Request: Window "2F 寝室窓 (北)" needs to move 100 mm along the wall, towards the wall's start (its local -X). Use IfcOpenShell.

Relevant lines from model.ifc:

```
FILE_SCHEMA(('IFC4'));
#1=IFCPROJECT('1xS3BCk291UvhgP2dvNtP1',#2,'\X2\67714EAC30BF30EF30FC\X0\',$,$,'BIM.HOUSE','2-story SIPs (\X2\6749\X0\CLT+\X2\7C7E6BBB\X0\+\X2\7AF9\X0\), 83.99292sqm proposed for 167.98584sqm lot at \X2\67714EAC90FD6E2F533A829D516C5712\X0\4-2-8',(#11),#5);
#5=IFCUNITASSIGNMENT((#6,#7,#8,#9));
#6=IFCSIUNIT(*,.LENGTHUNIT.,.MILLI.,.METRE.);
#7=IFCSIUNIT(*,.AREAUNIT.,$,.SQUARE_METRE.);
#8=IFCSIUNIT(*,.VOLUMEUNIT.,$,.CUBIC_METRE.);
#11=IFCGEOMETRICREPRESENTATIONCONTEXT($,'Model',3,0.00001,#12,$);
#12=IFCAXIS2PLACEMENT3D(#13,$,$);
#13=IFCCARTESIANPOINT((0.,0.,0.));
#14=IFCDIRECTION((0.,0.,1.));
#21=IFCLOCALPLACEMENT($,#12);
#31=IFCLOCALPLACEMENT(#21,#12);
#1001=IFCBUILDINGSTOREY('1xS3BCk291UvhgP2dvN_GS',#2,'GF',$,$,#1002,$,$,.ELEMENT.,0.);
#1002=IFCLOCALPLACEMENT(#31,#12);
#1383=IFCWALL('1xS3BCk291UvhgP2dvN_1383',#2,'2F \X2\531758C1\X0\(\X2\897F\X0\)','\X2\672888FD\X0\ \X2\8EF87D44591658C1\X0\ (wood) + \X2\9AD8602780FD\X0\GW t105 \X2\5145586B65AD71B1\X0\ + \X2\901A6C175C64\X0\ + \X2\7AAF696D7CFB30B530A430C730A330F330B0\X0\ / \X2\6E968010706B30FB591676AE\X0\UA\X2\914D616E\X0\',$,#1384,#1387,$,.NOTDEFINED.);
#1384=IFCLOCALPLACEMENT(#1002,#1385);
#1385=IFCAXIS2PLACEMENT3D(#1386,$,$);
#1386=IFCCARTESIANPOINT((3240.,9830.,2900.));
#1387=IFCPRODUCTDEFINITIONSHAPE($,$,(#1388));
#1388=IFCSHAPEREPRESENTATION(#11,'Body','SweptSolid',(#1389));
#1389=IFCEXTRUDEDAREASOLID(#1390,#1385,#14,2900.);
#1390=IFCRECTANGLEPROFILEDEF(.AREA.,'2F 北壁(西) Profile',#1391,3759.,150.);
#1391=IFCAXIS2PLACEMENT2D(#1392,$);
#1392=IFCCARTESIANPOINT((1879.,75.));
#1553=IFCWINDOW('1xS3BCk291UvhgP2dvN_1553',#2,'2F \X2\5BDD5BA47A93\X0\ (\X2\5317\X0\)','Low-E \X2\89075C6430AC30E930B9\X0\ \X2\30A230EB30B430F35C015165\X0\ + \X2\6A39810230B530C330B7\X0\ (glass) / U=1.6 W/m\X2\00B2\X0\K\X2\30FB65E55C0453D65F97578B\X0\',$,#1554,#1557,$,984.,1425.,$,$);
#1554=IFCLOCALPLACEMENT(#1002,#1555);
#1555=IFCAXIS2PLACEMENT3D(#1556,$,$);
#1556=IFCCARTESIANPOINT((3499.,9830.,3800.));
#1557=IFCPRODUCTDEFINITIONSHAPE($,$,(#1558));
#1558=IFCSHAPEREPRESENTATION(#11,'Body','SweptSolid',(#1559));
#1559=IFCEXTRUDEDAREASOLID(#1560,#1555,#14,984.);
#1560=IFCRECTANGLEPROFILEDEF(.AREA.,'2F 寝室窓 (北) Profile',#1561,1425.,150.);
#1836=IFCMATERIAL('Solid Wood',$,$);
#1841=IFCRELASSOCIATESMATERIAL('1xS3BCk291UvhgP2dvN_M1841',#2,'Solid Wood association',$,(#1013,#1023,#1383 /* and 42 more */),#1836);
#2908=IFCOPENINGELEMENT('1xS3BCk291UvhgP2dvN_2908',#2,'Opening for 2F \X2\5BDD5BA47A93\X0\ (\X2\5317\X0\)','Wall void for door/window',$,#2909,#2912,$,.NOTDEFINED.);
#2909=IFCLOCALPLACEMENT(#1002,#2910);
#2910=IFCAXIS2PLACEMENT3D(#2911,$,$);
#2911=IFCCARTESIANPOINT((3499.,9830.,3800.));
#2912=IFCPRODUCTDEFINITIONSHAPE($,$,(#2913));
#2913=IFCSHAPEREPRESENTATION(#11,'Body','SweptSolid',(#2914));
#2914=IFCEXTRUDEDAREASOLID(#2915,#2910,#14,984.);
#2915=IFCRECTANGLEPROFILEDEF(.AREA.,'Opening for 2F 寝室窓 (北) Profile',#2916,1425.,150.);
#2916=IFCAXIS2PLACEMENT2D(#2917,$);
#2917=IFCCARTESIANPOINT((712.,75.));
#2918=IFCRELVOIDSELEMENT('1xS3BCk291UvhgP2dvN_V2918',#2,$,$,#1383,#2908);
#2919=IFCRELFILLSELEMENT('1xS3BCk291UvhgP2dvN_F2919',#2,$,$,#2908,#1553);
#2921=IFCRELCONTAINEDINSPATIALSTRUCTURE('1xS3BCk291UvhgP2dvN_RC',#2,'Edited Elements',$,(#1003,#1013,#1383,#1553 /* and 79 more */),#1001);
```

```python
import ifcopenshell
import ifcopenshell.api.geometry
import ifcopenshell.util.placement

model = ifcopenshell.open("model.ifc")

window = model.by_id(1553)
opening = window.FillsVoids[0].RelatingOpeningElement
wall = opening.VoidsElements[0].RelatingBuildingElement

wall_matrix = ifcopenshell.util.placement.get_local_placement(wall.ObjectPlacement)
shift = wall_matrix[:3, 0] * -100.0
before = ifcopenshell.util.placement.get_local_placement(window.ObjectPlacement)[:3, 3].copy()

# The window is not placed relative to its opening, so move both.
for product in (opening, window):
    matrix = ifcopenshell.util.placement.get_local_placement(product.ObjectPlacement)
    matrix[:3, 3] += shift
    ifcopenshell.api.geometry.edit_object_placement(model, product=product, matrix=matrix, is_si=False)

after = ifcopenshell.util.placement.get_local_placement(window.ObjectPlacement)[:3, 3]
print("window moved by", (after - before).round(3) + 0.0)

model.write("model_rev.ifc")
```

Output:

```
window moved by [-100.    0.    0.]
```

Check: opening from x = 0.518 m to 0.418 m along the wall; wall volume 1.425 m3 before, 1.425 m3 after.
